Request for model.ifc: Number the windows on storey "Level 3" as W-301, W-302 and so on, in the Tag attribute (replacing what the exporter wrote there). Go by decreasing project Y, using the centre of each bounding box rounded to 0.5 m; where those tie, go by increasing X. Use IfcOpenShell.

First a look at what the model holds.

```python
import ifcopenshell
import ifcopenshell.util.element
import ifcopenshell.util.placement

model = ifcopenshell.open("model.ifc")
print(model.schema)
storey = next(s for s in model.by_type("IfcBuildingStorey") if s.Name == "Level 3")
windows = [e for e in ifcopenshell.util.element.get_decomposition(storey) if e.is_a("IfcWindow")]
for e in sorted(windows, key=lambda e: e.id()):
    origin = ifcopenshell.util.placement.get_local_placement(e.ObjectPlacement)[:3, 3]
    print(e.id(), e.Tag, e.Name, origin.round(2) + 0.0, sep=" | ")
```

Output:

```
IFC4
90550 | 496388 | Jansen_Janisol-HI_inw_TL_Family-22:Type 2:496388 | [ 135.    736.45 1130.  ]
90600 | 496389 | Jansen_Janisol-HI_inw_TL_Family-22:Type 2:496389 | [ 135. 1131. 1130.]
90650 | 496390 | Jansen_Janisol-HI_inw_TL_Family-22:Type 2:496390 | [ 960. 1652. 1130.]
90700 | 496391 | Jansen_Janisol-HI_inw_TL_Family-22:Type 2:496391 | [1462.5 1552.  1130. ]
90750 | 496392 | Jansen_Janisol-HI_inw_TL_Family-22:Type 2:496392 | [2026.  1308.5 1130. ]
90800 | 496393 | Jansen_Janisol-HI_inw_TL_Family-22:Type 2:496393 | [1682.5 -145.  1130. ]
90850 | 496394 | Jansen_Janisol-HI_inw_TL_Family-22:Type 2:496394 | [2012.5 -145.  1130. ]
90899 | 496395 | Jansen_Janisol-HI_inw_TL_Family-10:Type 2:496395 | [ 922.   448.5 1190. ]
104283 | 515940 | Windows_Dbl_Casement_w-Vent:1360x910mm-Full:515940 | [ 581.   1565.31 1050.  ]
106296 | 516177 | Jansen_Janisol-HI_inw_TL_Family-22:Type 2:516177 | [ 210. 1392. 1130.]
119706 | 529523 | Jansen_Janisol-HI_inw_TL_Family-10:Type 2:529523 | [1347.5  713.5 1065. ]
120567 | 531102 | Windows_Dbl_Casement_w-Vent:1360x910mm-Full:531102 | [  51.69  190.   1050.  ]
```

```python
import ifcopenshell
import ifcopenshell.geom
import ifcopenshell.util.element
import ifcopenshell.util.shape

model = ifcopenshell.open("model.ifc")
settings = ifcopenshell.geom.settings()
settings.set("use-world-coords", True)


def centre(element):
    shape = ifcopenshell.geom.create_shape(settings, element)
    return ifcopenshell.util.shape.get_bbox_centroid(shape.geometry)


storey = next(s for s in model.by_type("IfcBuildingStorey") if s.Name == "Level 3")
windows = [e for e in ifcopenshell.util.element.get_decomposition(storey) if e.is_a("IfcWindow")]

# Insertion points can sit at a corner or the storey origin, so sort by the geometry (in metres).
centres = {e: centre(e) for e in windows}
windows.sort(key=lambda e: (-round(centres[e][1] / 0.5), centres[e][0]))

for i, e in enumerate(windows, start=1):
    number = f"W-3{i:02d}"
    e.Tag = number
    print(e.id(), number)

model.write("model_updated.ifc")
```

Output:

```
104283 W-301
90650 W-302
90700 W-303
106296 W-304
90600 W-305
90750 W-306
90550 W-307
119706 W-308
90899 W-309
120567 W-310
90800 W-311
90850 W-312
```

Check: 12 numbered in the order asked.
